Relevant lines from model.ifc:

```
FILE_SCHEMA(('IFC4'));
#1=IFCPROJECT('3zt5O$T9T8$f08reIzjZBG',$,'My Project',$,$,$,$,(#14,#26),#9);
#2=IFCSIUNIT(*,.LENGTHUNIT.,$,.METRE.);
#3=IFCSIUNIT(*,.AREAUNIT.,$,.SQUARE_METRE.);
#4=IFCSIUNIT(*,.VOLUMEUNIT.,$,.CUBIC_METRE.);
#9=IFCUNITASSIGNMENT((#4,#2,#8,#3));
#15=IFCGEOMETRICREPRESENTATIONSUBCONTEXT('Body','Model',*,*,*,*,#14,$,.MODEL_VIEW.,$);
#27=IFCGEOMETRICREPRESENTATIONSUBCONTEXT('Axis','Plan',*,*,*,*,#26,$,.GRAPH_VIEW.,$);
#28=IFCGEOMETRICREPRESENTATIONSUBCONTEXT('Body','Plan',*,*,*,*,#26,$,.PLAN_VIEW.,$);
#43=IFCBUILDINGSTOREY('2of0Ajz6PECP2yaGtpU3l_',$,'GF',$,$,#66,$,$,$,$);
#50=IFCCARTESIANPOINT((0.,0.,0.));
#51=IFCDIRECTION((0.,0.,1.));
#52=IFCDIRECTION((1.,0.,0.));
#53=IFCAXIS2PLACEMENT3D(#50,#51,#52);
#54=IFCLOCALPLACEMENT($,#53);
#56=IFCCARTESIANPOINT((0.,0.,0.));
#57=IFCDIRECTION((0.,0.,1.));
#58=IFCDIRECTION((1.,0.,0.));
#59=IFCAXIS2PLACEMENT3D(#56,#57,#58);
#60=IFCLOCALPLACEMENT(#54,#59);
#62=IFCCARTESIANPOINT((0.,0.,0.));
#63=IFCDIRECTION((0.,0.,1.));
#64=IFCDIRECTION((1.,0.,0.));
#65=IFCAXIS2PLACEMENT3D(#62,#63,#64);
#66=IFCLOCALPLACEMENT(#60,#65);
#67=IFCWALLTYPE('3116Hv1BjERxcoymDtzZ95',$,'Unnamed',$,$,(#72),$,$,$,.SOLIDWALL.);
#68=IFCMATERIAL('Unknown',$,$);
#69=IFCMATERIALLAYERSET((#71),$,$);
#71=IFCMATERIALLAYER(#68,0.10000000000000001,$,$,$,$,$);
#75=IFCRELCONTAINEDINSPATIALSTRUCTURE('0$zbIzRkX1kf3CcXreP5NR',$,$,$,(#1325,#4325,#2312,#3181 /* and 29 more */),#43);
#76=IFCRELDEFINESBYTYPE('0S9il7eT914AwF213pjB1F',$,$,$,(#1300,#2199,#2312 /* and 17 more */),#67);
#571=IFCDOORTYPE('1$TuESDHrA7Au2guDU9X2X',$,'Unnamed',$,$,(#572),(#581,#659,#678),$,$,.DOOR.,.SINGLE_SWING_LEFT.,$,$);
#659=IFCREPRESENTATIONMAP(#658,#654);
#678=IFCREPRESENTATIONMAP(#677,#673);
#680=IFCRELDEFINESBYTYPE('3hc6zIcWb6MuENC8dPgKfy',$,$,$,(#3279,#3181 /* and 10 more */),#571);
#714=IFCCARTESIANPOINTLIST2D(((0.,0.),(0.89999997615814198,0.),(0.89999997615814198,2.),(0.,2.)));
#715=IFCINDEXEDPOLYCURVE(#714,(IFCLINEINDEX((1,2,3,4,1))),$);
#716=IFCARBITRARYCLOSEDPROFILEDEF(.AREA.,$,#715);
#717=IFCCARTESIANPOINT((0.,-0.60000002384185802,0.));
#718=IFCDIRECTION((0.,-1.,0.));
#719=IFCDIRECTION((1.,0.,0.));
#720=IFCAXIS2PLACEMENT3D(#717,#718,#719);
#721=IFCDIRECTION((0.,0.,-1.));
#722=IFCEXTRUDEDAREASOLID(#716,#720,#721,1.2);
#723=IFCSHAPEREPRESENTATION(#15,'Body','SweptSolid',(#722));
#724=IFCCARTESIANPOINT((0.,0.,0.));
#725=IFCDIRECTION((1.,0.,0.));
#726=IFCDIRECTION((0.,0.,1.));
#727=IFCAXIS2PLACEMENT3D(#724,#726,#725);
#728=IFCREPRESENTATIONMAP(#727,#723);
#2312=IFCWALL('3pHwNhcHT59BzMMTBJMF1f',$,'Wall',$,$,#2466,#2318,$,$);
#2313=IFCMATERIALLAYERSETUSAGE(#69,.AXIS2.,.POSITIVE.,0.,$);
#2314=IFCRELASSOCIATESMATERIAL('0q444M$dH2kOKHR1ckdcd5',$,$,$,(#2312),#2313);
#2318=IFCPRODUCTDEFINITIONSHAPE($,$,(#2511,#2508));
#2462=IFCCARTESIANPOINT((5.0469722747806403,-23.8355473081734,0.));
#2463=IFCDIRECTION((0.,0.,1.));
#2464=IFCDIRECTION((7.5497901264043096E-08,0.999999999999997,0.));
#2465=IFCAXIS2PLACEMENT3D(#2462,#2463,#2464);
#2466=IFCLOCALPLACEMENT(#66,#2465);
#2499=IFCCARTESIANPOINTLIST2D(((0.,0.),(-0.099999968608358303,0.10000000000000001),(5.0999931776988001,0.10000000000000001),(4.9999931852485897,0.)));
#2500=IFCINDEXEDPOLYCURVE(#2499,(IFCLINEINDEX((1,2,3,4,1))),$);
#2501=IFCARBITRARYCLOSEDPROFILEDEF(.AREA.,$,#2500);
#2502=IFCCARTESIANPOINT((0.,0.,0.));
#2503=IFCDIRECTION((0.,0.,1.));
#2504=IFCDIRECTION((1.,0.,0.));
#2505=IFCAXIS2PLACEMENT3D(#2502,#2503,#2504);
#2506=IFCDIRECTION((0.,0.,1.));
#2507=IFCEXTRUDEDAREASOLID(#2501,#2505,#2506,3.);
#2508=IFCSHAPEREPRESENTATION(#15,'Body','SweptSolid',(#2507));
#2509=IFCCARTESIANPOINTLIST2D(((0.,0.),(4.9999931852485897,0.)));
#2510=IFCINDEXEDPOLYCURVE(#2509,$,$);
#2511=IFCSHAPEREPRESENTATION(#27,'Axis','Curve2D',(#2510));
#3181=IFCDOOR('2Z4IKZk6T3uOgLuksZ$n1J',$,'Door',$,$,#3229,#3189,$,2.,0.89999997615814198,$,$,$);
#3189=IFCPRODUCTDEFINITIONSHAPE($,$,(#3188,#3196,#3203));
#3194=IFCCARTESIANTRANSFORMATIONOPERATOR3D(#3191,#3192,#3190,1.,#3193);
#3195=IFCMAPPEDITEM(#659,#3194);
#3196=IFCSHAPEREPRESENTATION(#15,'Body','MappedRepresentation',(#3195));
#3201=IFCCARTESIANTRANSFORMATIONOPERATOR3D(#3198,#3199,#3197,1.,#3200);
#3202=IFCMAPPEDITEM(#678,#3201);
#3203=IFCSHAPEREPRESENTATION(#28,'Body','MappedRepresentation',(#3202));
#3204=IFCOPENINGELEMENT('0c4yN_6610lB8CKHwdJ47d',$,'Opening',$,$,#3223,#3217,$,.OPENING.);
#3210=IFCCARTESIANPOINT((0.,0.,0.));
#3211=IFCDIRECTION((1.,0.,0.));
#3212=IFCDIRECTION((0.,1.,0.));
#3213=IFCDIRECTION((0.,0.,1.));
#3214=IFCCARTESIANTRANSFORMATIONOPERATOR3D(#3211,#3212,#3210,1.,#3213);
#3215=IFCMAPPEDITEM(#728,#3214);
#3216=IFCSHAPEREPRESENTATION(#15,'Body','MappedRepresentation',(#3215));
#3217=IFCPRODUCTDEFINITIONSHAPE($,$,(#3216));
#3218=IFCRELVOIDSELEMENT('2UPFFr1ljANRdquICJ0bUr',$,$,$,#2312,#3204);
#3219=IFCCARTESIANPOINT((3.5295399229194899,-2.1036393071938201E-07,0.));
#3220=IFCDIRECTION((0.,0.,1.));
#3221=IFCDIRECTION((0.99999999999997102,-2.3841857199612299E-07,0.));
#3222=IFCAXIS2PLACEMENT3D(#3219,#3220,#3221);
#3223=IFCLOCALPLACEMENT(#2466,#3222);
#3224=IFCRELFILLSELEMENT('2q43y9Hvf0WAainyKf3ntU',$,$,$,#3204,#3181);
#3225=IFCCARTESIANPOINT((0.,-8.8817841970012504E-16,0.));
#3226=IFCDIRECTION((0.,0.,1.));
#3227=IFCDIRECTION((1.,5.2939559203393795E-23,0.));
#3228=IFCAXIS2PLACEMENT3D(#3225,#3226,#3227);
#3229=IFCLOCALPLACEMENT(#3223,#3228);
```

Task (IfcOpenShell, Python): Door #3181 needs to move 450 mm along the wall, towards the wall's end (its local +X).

```python
import ifcopenshell
import ifcopenshell.api.geometry
import ifcopenshell.util.placement

model = ifcopenshell.open("model.ifc")

door = model.by_guid("2Z4IKZk6T3uOgLuksZ$n1J")
opening = door.FillsVoids[0].RelatingOpeningElement
wall = opening.VoidsElements[0].RelatingBuildingElement

wall_matrix = ifcopenshell.util.placement.get_local_placement(wall.ObjectPlacement)
shift = wall_matrix[:3, 0] * 0.45
before = ifcopenshell.util.placement.get_local_placement(door.ObjectPlacement)[:3, 3].copy()

# The door is placed relative to its opening, so it follows when the opening moves.
matrix = ifcopenshell.util.placement.get_local_placement(opening.ObjectPlacement)
matrix[:3, 3] += shift
ifcopenshell.api.geometry.edit_object_placement(
    model, product=opening, matrix=matrix, is_si=False, should_transform_children=True
)

after = ifcopenshell.util.placement.get_local_placement(door.ObjectPlacement)[:3, 3]
print("door moved by", (after - before).round(3) + 0.0)

model.write("model_edited.ifc")
```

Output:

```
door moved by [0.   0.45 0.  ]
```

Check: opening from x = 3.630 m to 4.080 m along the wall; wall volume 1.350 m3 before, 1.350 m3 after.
